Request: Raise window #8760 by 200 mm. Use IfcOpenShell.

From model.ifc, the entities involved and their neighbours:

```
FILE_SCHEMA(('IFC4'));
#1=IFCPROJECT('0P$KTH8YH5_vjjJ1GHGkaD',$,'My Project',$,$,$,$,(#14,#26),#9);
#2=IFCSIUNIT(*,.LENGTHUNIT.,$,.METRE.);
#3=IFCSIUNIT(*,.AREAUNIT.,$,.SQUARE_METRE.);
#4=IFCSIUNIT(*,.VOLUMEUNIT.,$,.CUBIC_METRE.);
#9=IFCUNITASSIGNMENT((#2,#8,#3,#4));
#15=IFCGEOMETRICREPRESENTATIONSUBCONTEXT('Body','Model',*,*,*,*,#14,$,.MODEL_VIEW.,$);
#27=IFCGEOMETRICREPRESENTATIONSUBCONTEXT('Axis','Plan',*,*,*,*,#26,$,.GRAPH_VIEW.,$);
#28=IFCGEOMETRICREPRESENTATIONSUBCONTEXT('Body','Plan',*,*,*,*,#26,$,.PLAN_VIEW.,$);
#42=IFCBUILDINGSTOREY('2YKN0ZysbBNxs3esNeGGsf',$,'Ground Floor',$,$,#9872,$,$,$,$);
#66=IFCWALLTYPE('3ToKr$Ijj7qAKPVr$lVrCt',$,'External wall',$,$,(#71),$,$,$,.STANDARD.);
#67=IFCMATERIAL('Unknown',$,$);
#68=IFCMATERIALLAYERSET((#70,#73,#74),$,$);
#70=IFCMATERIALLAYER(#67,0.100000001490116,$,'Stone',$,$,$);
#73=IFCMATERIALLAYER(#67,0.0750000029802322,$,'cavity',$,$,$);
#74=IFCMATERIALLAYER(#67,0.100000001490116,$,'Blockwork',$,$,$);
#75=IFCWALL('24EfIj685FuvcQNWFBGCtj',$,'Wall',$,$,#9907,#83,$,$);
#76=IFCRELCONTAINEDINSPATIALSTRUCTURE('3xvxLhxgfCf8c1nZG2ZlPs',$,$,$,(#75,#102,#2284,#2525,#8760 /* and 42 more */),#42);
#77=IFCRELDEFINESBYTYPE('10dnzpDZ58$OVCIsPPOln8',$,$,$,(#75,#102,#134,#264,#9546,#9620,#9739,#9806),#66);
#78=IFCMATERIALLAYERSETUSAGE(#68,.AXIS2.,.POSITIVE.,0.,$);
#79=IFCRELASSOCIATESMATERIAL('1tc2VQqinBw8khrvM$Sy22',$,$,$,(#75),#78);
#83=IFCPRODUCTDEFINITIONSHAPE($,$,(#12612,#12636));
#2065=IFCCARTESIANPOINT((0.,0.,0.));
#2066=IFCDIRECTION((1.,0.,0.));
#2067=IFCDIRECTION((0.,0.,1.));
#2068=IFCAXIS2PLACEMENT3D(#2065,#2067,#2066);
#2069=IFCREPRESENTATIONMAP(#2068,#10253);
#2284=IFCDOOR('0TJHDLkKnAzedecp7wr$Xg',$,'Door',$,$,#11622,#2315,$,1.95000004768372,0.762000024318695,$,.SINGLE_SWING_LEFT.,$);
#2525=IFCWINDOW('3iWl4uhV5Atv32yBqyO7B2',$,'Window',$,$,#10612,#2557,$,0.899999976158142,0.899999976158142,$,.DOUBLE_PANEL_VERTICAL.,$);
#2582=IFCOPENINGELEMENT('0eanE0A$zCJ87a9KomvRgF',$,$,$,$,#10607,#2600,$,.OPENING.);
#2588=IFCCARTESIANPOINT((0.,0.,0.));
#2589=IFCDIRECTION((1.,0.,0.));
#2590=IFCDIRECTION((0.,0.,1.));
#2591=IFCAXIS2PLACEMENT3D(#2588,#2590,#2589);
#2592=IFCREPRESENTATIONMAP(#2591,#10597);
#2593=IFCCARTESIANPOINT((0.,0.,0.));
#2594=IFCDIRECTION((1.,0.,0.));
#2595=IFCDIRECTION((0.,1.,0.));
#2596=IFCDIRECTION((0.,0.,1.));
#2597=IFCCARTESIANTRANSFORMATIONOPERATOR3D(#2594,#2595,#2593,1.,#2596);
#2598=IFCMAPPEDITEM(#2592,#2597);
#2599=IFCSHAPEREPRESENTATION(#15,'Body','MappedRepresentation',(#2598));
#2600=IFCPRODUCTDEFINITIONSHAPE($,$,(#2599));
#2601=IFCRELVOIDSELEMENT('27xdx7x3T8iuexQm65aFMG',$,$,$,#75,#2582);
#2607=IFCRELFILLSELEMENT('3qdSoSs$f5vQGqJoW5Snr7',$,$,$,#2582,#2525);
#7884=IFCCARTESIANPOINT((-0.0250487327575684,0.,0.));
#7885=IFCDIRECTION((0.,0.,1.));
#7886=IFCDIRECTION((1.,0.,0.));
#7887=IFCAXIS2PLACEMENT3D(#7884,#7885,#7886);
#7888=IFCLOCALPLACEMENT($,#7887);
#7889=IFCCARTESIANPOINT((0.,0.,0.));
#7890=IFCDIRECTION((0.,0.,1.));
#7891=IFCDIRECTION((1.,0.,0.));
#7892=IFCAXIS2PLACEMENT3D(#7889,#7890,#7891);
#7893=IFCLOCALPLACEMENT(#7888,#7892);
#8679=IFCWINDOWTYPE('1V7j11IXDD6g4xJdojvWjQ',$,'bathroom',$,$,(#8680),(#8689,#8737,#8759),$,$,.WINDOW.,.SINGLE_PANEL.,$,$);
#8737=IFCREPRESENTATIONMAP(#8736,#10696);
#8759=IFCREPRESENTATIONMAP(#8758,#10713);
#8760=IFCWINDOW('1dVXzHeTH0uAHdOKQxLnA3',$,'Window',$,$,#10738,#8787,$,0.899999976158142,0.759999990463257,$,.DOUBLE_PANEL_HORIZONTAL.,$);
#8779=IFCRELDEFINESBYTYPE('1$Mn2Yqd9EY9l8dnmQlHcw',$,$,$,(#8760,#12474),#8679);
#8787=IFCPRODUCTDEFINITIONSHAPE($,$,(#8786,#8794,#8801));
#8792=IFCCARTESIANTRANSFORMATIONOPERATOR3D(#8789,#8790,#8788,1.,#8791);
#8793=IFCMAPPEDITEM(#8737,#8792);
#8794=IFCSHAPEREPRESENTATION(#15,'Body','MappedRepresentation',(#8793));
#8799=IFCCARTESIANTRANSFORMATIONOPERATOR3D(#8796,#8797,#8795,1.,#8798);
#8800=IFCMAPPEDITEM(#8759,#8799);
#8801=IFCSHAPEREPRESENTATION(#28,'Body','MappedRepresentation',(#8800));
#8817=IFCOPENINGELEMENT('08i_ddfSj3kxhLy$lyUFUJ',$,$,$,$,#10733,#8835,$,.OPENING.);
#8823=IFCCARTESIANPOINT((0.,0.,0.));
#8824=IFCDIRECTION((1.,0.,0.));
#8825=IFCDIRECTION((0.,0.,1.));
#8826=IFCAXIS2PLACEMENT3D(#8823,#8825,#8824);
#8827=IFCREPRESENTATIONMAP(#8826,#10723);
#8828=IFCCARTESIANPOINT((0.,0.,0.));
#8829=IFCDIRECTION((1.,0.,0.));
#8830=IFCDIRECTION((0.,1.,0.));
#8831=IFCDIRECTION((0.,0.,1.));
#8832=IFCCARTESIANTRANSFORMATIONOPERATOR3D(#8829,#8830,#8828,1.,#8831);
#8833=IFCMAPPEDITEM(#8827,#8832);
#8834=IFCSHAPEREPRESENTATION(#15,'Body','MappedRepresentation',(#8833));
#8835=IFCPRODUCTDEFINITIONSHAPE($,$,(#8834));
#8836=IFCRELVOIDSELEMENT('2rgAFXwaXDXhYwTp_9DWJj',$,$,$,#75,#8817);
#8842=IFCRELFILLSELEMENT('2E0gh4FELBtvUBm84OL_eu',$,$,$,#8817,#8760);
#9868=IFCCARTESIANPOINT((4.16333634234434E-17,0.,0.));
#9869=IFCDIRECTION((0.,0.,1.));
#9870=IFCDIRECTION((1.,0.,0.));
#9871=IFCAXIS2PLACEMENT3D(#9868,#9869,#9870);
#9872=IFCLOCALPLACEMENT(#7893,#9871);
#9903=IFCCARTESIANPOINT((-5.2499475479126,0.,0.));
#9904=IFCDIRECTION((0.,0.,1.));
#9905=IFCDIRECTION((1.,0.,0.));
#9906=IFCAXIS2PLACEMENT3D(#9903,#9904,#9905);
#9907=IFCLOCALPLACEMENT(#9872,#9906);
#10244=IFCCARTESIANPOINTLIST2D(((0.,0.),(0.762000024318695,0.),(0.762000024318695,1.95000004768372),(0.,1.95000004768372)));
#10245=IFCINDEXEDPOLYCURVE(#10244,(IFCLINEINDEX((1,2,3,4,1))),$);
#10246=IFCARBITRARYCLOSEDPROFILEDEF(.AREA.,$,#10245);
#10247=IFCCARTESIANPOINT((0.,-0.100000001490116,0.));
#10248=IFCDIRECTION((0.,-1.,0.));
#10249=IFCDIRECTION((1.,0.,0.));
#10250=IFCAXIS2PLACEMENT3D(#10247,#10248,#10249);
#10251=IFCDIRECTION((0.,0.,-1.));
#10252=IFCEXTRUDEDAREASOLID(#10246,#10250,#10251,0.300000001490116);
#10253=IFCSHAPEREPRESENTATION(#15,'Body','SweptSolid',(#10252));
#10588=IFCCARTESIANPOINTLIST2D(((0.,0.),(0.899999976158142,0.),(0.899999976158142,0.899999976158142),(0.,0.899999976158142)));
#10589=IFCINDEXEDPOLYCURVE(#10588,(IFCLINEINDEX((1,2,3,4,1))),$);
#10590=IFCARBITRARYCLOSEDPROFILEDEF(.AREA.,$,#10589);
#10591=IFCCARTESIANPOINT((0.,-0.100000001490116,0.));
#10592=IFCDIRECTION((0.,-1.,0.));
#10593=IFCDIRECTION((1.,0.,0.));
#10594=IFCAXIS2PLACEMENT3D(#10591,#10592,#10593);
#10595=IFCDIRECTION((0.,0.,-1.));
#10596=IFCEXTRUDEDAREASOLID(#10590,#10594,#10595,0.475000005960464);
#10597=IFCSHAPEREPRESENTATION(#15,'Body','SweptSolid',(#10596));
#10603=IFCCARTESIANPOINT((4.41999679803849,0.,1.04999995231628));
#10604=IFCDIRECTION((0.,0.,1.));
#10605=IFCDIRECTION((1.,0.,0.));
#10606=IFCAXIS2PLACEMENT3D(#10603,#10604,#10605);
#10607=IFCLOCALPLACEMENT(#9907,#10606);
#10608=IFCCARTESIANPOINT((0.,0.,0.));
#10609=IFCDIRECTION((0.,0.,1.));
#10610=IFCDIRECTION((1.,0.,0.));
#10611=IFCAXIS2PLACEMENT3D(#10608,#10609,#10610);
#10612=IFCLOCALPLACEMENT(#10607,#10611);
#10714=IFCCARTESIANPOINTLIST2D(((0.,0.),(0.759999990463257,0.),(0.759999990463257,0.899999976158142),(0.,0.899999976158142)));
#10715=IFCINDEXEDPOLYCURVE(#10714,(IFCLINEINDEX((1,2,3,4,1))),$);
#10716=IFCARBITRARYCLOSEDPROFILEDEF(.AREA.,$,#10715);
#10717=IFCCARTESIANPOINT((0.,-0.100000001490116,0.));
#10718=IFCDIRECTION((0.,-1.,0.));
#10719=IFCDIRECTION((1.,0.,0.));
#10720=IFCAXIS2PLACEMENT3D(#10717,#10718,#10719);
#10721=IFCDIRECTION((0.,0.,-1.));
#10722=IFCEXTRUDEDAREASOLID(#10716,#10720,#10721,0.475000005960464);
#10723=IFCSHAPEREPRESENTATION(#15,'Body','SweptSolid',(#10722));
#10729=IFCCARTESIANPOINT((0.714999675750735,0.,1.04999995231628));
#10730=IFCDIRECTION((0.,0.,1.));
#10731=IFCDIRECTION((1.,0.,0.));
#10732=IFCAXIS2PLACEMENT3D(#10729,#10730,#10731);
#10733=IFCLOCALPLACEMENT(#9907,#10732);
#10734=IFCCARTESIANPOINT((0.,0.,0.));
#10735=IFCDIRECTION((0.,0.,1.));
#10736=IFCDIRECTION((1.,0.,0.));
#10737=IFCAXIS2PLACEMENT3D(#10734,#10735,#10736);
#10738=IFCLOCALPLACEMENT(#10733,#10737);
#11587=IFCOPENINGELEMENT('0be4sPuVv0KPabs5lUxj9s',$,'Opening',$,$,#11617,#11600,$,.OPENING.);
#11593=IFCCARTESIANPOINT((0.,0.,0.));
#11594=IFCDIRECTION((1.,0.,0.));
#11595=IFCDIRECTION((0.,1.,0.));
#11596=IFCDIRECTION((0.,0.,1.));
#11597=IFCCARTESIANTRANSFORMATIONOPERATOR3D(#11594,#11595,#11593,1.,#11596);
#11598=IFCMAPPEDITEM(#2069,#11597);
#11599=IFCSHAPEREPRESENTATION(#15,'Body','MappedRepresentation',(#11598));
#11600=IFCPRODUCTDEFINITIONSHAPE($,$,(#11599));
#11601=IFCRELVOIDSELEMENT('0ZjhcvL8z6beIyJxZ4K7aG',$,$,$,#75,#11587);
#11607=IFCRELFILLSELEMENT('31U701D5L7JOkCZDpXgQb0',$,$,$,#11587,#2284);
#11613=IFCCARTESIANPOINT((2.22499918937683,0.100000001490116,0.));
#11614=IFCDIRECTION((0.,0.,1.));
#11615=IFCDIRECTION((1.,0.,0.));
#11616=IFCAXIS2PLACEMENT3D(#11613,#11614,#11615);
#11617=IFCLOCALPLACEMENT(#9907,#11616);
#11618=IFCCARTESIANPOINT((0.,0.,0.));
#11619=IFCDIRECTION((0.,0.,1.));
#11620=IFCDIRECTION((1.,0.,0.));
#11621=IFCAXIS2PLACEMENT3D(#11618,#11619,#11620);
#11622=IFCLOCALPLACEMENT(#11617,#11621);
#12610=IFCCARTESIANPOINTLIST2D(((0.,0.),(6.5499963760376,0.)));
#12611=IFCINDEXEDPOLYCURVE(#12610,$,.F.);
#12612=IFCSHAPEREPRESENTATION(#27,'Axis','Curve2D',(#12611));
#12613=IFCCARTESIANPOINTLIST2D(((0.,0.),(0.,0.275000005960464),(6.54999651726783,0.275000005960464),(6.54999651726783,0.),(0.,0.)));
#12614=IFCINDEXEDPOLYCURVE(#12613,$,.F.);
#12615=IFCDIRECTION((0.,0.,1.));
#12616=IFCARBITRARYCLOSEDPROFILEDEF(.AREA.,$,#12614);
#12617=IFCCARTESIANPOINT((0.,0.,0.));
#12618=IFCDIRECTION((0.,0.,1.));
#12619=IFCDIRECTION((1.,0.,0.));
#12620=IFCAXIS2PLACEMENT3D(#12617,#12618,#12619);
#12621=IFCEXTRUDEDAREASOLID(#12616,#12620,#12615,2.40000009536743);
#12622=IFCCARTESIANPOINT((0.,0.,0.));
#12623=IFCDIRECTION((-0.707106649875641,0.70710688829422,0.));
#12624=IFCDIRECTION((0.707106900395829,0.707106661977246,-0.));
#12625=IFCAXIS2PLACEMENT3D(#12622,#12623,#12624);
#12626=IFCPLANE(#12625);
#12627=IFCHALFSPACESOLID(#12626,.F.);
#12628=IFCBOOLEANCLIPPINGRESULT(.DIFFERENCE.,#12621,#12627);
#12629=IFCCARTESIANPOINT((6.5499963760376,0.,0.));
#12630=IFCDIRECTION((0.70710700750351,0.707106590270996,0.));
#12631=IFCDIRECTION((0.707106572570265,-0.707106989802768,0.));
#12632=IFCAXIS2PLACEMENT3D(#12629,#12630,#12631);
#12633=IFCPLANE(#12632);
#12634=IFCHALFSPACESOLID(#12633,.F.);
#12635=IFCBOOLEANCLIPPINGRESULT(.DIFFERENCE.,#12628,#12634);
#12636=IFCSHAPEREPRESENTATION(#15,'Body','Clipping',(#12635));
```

```python
import numpy as np
import ifcopenshell
import ifcopenshell.api.geometry
import ifcopenshell.util.placement
import ifcopenshell.util.unit

model = ifcopenshell.open("model.ifc")
unit_scale = ifcopenshell.util.unit.calculate_unit_scale(model)

window = model.by_guid("1dVXzHeTH0uAHdOKQxLnA3")
opening = window.FillsVoids[0].RelatingOpeningElement
dz = 0.2 / unit_scale

shift = np.array([0.0, 0.0, dz])
# The window is placed relative to its opening, so it follows when the opening moves.
matrix = ifcopenshell.util.placement.get_local_placement(opening.ObjectPlacement)
matrix[:3, 3] += shift
ifcopenshell.api.geometry.edit_object_placement(
    model, product=opening, matrix=matrix, is_si=False, should_transform_children=True
)

print(f"moved by {dz * unit_scale:+.3f} m")

model.write("model_updated.ifc")
```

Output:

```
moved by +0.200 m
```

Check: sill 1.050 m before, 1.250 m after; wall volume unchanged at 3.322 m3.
